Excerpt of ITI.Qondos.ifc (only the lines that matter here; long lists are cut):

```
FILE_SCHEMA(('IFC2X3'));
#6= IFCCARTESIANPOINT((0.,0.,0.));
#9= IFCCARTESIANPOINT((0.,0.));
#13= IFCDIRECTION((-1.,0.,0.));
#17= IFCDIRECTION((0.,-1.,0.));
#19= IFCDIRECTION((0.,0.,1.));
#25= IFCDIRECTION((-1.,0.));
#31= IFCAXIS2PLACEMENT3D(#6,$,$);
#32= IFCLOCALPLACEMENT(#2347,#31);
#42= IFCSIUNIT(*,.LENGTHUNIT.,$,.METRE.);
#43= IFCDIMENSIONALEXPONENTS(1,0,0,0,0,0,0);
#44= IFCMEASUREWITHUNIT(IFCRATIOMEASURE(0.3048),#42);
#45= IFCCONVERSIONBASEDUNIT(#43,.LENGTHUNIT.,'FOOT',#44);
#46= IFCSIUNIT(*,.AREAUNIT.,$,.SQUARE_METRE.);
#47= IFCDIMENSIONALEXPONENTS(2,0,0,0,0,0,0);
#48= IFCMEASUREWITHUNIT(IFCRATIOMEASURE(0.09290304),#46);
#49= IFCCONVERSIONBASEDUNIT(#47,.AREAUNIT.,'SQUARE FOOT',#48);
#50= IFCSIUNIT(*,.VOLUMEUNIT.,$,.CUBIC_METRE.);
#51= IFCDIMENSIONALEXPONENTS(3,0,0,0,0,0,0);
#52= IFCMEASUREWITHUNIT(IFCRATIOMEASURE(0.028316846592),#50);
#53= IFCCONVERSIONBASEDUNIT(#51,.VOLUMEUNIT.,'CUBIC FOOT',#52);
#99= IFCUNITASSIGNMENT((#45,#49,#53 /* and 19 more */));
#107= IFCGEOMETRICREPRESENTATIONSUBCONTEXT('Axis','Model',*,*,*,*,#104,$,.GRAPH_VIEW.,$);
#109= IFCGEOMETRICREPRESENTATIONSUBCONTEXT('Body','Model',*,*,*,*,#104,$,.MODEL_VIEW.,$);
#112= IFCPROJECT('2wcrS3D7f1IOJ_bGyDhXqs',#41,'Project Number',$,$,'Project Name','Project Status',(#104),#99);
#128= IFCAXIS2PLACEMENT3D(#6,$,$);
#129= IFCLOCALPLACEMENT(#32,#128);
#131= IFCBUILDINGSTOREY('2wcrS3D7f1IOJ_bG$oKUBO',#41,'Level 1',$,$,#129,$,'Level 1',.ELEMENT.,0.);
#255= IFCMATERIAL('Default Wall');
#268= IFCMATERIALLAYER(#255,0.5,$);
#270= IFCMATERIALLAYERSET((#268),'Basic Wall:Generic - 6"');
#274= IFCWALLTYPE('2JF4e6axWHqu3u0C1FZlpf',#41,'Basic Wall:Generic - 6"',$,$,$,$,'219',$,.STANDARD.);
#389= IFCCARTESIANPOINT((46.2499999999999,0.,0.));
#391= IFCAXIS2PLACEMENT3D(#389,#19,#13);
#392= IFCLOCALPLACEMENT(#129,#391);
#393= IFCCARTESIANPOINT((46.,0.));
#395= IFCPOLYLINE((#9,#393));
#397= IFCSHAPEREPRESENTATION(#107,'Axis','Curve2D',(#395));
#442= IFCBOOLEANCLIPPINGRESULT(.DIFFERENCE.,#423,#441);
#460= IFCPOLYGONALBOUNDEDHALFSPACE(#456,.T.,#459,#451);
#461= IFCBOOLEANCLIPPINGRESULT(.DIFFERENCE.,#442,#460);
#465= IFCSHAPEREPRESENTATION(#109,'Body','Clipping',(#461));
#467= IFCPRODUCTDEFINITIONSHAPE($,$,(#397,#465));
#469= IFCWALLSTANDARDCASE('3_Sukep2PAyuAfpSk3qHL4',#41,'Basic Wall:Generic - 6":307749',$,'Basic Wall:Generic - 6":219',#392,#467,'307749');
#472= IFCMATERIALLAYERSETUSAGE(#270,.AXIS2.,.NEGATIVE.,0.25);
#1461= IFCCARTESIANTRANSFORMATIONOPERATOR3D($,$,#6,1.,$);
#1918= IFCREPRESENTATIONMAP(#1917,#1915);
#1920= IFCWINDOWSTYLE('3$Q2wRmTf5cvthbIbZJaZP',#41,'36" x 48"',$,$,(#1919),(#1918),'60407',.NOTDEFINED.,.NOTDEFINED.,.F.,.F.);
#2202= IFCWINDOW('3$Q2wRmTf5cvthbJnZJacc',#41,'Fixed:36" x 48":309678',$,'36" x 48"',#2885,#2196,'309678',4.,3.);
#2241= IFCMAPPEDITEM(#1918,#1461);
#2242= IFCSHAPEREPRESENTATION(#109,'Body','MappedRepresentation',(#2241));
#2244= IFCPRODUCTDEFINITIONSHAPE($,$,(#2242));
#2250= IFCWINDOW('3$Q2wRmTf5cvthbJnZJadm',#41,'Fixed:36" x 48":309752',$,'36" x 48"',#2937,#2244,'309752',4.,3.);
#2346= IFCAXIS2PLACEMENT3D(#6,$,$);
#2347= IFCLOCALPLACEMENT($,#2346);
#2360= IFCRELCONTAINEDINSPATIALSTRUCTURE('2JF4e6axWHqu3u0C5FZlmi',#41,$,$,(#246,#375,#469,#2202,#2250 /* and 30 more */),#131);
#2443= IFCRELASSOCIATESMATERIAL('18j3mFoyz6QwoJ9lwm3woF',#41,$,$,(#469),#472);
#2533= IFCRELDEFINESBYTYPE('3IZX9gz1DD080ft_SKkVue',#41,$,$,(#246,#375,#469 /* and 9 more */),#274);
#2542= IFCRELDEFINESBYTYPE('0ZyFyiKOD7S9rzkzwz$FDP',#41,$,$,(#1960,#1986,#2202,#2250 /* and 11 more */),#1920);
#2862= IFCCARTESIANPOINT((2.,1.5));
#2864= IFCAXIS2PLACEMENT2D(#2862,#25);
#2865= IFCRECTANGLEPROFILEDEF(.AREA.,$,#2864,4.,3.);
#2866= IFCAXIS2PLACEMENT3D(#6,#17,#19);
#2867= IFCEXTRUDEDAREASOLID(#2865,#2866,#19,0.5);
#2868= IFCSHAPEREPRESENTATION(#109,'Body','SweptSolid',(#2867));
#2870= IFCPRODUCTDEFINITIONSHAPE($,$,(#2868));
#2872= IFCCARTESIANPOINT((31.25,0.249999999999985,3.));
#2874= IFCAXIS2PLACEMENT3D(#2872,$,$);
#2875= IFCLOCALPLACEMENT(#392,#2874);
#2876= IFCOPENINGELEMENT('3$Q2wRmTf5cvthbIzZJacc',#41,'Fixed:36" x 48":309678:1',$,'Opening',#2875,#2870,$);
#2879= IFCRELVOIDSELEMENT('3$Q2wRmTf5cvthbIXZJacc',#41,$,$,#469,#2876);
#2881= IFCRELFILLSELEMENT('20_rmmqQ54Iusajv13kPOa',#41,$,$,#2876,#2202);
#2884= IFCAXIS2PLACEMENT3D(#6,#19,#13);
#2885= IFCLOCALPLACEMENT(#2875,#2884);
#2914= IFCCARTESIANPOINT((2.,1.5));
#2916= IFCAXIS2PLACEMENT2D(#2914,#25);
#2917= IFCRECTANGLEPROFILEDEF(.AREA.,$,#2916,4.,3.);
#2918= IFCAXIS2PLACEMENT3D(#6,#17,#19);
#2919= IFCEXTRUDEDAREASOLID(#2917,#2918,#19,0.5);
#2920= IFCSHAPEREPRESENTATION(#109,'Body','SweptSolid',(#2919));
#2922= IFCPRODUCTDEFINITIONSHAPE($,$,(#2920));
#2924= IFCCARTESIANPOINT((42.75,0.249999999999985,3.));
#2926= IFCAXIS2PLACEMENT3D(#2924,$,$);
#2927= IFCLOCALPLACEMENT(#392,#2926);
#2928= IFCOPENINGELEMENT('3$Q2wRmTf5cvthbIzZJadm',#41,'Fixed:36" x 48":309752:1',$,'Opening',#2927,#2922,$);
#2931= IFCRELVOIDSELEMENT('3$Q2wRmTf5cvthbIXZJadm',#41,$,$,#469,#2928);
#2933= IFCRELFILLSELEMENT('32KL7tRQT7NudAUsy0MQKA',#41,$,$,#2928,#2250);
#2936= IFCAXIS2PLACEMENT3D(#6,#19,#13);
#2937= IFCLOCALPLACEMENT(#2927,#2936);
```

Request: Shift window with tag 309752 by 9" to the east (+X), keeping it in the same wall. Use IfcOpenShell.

```python
import ifcopenshell
import ifcopenshell.api.geometry
import ifcopenshell.util.placement
import ifcopenshell.util.unit

model = ifcopenshell.open("ITI.Qondos.ifc")
unit_scale = ifcopenshell.util.unit.calculate_unit_scale(model)

window = model.by_id(2250)
opening = window.FillsVoids[0].RelatingOpeningElement
wall = opening.VoidsElements[0].RelatingBuildingElement

wall_matrix = ifcopenshell.util.placement.get_local_placement(wall.ObjectPlacement)
shift = wall_matrix[:3, 0] * -9 * 0.0254 / unit_scale
before = ifcopenshell.util.placement.get_local_placement(window.ObjectPlacement)[:3, 3].copy()

# The window is placed relative to its opening, so it follows when the opening moves.
matrix = ifcopenshell.util.placement.get_local_placement(opening.ObjectPlacement)
matrix[:3, 3] += shift
ifcopenshell.api.geometry.edit_object_placement(
    model, product=opening, matrix=matrix, is_si=False, should_transform_children=True
)

after = ifcopenshell.util.placement.get_local_placement(window.ObjectPlacement)[:3, 3]
print("window moved by", (after - before).round(3) + 0.0)

model.write("ITI.Qondos_rev.ifc")
```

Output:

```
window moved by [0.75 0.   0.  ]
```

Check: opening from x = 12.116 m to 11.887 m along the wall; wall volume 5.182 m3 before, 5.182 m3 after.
